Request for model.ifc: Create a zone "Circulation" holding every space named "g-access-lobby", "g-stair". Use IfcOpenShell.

First a look at what the model holds.

```python
import ifcopenshell

model = ifcopenshell.open("model.ifc")
print(model.schema)
seen = {}
for space in model.by_type("IfcSpace"):
    seen[space.LongName] = seen.get(space.LongName, 0) + 1
for name, count in sorted(seen.items(), key=str):
    print(count, "x", name)
print("zones:", [z.Name for z in model.by_type("IfcZone")][:20])
```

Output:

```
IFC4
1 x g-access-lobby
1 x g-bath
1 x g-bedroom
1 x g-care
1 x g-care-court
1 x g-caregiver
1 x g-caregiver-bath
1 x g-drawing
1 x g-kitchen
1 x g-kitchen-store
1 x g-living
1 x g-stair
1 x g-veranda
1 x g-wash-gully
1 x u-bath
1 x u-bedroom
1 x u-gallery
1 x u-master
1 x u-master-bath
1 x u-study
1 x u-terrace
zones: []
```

```python
import ifcopenshell
import ifcopenshell.api.group
import ifcopenshell.api.root

model = ifcopenshell.open("model.ifc")

names = {"g-access-lobby", "g-stair"}
spaces = [s for s in model.by_type("IfcSpace") if s.LongName in names]

zone = ifcopenshell.api.root.create_entity(model, ifc_class="IfcZone", name="Circulation")
ifcopenshell.api.group.assign_group(model, products=spaces, group=zone)
print(len(spaces), "spaces in", zone.Name)

model.write("model-out.ifc")
```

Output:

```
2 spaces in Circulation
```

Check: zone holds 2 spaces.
